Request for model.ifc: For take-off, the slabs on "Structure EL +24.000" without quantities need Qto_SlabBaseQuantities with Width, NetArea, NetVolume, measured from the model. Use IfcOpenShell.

First a look at what the model holds.

```python
import ifcopenshell
import ifcopenshell.util.element
import ifcopenshell.util.unit

model = ifcopenshell.open("model.ifc")
print(model.schema)
for unit_type in ("LENGTHUNIT", "AREAUNIT", "VOLUMEUNIT"):
    print(unit_type, ifcopenshell.util.unit.calculate_unit_scale(model, unit_type))
storey = next(s for s in model.by_type("IfcBuildingStorey") if s.Name == "Structure EL +24.000")
slabs = [e for e in ifcopenshell.util.element.get_decomposition(storey) if e.is_a("IfcSlab")]
for e in sorted(slabs, key=lambda e: e.id()):
    print(e.id(), e.is_a(), e.Name, list(ifcopenshell.util.element.get_psets(e, qtos_only=True)), sep=" | ")
```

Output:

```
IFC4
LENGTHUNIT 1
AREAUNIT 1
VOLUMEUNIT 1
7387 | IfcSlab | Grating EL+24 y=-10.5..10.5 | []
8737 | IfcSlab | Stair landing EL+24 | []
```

```python
import ifcopenshell
import ifcopenshell.api.pset
import ifcopenshell.geom
import ifcopenshell.util.element
import ifcopenshell.util.shape
import ifcopenshell.util.unit

model = ifcopenshell.open("model.ifc")
unit_scale = ifcopenshell.util.unit.calculate_unit_scale(model)
area_scale = ifcopenshell.util.unit.calculate_unit_scale(model, "AREAUNIT")
volume_scale = ifcopenshell.util.unit.calculate_unit_scale(model, "VOLUMEUNIT")
settings = ifcopenshell.geom.settings()

storey = next(s for s in model.by_type("IfcBuildingStorey") if s.Name == "Structure EL +24.000")
slabs = [e for e in ifcopenshell.util.element.get_decomposition(storey) if e.is_a("IfcSlab")]

for e in sorted(slabs, key=lambda e: e.id()):
    if ifcopenshell.util.element.get_psets(e, qtos_only=True, should_inherit=False):
        continue
    # Geometry comes back in metres, in the element's own axes.
    shape = ifcopenshell.geom.create_shape(settings, e)
    values = {
        "Width": ifcopenshell.util.shape.get_z(shape.geometry) / unit_scale,
        "NetArea": ifcopenshell.util.shape.get_footprint_area(shape.geometry) / area_scale,
        "NetVolume": ifcopenshell.util.shape.get_volume(shape.geometry) / volume_scale,
    }
    qto = ifcopenshell.api.pset.add_qto(model, product=e, name="Qto_SlabBaseQuantities")
    ifcopenshell.api.pset.edit_qto(model, qto=qto, properties=values)
    print(e.id(), {k: round(v, 3) for k, v in values.items()})

model.write("model_v2.ifc")
```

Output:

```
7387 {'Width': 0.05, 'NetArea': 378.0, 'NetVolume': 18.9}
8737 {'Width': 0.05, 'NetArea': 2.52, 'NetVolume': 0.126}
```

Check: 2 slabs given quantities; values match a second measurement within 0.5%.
